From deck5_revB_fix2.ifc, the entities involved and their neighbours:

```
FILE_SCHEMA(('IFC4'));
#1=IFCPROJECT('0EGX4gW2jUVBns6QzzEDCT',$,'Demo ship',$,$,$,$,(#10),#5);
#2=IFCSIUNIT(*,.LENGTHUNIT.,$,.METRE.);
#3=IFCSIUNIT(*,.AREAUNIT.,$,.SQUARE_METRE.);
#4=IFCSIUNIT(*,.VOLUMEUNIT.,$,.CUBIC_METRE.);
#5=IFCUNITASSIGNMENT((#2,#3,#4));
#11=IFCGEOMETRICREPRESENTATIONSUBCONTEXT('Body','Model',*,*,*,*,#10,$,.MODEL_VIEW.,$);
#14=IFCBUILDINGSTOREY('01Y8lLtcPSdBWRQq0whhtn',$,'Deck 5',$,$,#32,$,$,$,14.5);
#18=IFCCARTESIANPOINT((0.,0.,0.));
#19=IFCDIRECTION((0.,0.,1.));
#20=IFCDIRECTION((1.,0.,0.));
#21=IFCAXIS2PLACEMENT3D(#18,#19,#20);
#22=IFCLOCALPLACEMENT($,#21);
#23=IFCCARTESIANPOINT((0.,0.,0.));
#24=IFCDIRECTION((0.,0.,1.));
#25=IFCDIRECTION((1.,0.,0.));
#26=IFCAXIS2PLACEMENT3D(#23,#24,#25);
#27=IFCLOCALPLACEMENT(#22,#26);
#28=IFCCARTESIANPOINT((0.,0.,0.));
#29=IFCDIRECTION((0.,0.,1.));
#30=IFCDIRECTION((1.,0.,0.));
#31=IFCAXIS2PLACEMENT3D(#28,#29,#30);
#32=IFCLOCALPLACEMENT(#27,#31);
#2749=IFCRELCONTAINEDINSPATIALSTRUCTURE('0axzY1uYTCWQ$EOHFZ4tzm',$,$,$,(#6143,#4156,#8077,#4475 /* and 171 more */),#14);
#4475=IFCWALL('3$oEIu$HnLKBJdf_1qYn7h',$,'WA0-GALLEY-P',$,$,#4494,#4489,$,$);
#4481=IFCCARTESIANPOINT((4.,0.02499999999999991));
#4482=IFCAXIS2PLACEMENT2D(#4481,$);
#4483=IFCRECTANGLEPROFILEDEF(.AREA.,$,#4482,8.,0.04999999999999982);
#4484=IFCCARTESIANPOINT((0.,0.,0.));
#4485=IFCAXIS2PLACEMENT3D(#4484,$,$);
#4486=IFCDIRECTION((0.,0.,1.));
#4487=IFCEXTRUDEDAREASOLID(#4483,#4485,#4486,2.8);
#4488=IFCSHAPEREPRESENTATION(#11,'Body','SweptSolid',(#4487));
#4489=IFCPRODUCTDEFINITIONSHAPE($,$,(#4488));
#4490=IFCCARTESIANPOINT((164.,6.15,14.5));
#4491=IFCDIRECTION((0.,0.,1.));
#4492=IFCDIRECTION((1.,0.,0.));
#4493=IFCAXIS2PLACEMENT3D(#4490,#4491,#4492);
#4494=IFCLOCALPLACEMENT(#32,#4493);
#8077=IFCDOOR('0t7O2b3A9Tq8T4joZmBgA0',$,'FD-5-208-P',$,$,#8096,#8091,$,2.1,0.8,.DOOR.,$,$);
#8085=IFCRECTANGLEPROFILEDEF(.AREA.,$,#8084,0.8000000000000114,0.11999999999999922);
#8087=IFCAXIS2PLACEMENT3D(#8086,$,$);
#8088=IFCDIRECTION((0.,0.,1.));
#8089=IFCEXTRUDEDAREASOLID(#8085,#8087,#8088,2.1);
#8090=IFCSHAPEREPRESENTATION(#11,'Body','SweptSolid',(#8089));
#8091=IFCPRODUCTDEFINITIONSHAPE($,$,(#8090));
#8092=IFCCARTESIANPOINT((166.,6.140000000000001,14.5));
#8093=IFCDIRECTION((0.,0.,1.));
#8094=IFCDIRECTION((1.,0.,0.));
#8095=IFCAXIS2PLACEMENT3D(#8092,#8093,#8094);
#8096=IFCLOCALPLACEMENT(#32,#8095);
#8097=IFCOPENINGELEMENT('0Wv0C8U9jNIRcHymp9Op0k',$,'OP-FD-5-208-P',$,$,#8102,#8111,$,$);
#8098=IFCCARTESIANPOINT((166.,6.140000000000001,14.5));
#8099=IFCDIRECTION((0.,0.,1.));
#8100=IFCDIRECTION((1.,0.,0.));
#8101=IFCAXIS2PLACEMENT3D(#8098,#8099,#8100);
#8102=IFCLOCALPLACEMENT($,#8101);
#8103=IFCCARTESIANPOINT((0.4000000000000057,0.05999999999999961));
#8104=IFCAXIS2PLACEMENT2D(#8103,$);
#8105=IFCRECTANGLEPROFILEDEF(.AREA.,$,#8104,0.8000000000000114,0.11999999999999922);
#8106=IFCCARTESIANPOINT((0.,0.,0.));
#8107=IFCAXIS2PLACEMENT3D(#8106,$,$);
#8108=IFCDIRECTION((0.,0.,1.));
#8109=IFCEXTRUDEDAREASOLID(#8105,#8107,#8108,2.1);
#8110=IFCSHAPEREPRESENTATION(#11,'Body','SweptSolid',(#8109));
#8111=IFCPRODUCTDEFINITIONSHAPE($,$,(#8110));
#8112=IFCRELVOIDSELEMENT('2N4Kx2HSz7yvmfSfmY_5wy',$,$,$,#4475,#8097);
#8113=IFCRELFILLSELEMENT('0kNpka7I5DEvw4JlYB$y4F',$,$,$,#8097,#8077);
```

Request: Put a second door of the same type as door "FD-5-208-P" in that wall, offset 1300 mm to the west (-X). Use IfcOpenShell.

```python
import ifcopenshell
import ifcopenshell.api.feature
import ifcopenshell.api.geometry
import ifcopenshell.api.root
import ifcopenshell.geom
import ifcopenshell.util.element
import ifcopenshell.util.placement
import ifcopenshell.util.shape
import ifcopenshell.util.unit

model = ifcopenshell.open("deck5_revB_fix2.ifc")
unit_scale = ifcopenshell.util.unit.calculate_unit_scale(model)
settings = ifcopenshell.geom.settings()


def volume(element):
    """Net volume in cubic metres, openings subtracted."""
    shape = ifcopenshell.geom.create_shape(settings, element)
    return ifcopenshell.util.shape.get_volume(shape.geometry)


door = model.by_guid("0t7O2b3A9Tq8T4joZmBgA0")
opening = door.FillsVoids[0].RelatingOpeningElement
wall = opening.VoidsElements[0].RelatingBuildingElement
before = volume(wall)
shift = ifcopenshell.util.placement.get_local_placement(wall.ObjectPlacement)[:3, 0] * -1.3 / unit_scale

# copy_class copies the void relationship, type, container and properties, but no geometry.
new_opening = ifcopenshell.api.root.copy_class(model, product=opening)
new_opening.Representation = ifcopenshell.util.element.copy_deep(
    model, opening.Representation, exclude=["IfcGeometricRepresentationContext", "IfcRepresentationMap"]
)
new_door = ifcopenshell.api.root.copy_class(model, product=door)
new_door.Representation = ifcopenshell.util.element.copy_deep(
    model, door.Representation, exclude=["IfcGeometricRepresentationContext", "IfcRepresentationMap"]
)
ifcopenshell.api.feature.add_filling(model, opening=new_opening, element=new_door)

for old, new in ((opening, new_opening), (door, new_door)):
    matrix = ifcopenshell.util.placement.get_local_placement(old.ObjectPlacement)
    matrix[:3, 3] += shift
    ifcopenshell.api.geometry.edit_object_placement(model, product=new, matrix=matrix, is_si=False)

after = volume(wall)

print(f"wall volume {before:.3f} -> {after:.3f} m3")

model.write("deck5_revB_fix2_updated.ifc")
```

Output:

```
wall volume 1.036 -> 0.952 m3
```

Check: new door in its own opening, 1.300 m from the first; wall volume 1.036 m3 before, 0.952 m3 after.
